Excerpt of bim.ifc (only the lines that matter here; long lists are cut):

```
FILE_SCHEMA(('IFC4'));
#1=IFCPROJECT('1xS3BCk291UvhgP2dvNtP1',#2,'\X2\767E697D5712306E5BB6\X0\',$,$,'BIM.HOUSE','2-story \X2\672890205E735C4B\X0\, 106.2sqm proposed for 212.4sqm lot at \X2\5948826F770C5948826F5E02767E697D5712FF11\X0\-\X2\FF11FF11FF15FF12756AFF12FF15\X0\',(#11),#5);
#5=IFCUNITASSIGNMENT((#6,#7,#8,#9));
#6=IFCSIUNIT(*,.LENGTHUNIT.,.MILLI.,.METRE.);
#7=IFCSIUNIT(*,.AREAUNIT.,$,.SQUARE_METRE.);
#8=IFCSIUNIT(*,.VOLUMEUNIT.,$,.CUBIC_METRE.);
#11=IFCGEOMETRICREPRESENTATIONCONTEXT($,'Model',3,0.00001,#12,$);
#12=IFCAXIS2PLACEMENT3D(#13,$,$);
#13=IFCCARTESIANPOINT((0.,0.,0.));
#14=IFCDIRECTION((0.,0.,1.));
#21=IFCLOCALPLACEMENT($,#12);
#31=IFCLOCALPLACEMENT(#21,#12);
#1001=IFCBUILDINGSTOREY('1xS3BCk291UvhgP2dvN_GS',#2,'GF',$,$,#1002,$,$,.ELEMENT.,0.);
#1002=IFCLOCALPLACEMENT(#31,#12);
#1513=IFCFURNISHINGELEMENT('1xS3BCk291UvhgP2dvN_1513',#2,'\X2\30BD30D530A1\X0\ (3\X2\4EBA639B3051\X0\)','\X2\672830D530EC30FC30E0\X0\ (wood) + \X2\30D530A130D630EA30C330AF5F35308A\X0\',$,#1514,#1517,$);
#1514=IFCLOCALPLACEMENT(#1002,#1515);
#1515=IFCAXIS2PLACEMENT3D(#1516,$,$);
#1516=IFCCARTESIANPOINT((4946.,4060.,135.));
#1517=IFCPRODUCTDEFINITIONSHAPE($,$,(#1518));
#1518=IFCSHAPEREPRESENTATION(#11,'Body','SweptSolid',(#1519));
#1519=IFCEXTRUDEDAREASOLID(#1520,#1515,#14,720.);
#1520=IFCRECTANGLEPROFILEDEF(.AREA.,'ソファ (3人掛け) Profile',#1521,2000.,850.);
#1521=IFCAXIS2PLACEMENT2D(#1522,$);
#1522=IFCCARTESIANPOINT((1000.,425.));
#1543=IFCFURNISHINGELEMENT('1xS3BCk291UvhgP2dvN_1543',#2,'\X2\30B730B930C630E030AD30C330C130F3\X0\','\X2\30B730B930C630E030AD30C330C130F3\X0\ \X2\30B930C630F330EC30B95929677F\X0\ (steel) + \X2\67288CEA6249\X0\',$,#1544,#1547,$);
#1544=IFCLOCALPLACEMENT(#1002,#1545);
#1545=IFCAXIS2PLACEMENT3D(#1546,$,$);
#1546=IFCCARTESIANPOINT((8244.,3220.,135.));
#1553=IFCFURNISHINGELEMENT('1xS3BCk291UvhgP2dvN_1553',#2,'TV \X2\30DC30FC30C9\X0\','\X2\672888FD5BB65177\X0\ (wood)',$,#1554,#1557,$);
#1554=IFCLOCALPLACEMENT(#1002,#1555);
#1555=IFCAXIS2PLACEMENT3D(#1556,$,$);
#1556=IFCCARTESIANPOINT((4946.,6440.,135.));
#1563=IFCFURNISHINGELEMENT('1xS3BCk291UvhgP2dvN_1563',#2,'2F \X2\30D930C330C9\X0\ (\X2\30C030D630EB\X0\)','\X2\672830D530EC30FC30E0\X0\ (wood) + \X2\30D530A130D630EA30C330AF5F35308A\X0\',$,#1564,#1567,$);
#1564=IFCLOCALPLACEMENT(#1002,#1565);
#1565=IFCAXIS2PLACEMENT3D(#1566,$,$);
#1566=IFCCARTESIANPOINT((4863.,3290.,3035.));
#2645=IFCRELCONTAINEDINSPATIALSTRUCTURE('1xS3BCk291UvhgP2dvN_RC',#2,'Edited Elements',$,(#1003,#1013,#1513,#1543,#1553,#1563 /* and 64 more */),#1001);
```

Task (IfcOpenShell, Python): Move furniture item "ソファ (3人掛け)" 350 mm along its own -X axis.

```python
import ifcopenshell
import ifcopenshell.api.geometry
import ifcopenshell.util.placement
import ifcopenshell.util.unit

model = ifcopenshell.open("bim.ifc")
unit_scale = ifcopenshell.util.unit.calculate_unit_scale(model)

item = model.by_id(1513)
matrix = ifcopenshell.util.placement.get_local_placement(item.ObjectPlacement)
matrix[:3, 3] -= matrix[:3, 0] * 0.35 / unit_scale
ifcopenshell.api.geometry.edit_object_placement(model, product=item, matrix=matrix, is_si=False)

print(ifcopenshell.util.placement.get_local_placement(item.ObjectPlacement).round(3) + 0.0)

model.write("bim_edited.ifc")
```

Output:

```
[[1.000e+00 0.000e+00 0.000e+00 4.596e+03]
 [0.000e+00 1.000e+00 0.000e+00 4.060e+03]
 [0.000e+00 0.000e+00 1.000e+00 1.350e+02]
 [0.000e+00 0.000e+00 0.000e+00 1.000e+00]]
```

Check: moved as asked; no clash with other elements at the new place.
